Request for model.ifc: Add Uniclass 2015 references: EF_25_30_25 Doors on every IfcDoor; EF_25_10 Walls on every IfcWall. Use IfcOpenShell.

First a look at what the model holds.

```python
import ifcopenshell

model = ifcopenshell.open("model.ifc")
print(model.schema)
print("classifications:", [c.Name for c in model.by_type("IfcClassification")])
for ifc_class in ("IfcDoor", "IfcRoof", "IfcStair", "IfcWall", "IfcWindow"):
    print(ifc_class, len(model.by_type(ifc_class)))
```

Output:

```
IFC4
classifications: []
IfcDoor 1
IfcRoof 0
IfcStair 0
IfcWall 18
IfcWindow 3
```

```python
import ifcopenshell
import ifcopenshell.api.classification

model = ifcopenshell.open("model.ifc")

system = ifcopenshell.api.classification.add_classification(model, classification="Uniclass 2015")

codes = {
    "IfcDoor": ("EF_25_30_25", "Doors"),
    "IfcWall": ("EF_25_10", "Walls"),
}
for ifc_class, (code, name) in codes.items():
    products = model.by_type(ifc_class)
    ifcopenshell.api.classification.add_reference(
        model, products=products, classification=system, identification=code, name=name
    )
    print(code, len(products))

model.write("model_v2.ifc")
```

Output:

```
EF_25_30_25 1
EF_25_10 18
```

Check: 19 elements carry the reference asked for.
